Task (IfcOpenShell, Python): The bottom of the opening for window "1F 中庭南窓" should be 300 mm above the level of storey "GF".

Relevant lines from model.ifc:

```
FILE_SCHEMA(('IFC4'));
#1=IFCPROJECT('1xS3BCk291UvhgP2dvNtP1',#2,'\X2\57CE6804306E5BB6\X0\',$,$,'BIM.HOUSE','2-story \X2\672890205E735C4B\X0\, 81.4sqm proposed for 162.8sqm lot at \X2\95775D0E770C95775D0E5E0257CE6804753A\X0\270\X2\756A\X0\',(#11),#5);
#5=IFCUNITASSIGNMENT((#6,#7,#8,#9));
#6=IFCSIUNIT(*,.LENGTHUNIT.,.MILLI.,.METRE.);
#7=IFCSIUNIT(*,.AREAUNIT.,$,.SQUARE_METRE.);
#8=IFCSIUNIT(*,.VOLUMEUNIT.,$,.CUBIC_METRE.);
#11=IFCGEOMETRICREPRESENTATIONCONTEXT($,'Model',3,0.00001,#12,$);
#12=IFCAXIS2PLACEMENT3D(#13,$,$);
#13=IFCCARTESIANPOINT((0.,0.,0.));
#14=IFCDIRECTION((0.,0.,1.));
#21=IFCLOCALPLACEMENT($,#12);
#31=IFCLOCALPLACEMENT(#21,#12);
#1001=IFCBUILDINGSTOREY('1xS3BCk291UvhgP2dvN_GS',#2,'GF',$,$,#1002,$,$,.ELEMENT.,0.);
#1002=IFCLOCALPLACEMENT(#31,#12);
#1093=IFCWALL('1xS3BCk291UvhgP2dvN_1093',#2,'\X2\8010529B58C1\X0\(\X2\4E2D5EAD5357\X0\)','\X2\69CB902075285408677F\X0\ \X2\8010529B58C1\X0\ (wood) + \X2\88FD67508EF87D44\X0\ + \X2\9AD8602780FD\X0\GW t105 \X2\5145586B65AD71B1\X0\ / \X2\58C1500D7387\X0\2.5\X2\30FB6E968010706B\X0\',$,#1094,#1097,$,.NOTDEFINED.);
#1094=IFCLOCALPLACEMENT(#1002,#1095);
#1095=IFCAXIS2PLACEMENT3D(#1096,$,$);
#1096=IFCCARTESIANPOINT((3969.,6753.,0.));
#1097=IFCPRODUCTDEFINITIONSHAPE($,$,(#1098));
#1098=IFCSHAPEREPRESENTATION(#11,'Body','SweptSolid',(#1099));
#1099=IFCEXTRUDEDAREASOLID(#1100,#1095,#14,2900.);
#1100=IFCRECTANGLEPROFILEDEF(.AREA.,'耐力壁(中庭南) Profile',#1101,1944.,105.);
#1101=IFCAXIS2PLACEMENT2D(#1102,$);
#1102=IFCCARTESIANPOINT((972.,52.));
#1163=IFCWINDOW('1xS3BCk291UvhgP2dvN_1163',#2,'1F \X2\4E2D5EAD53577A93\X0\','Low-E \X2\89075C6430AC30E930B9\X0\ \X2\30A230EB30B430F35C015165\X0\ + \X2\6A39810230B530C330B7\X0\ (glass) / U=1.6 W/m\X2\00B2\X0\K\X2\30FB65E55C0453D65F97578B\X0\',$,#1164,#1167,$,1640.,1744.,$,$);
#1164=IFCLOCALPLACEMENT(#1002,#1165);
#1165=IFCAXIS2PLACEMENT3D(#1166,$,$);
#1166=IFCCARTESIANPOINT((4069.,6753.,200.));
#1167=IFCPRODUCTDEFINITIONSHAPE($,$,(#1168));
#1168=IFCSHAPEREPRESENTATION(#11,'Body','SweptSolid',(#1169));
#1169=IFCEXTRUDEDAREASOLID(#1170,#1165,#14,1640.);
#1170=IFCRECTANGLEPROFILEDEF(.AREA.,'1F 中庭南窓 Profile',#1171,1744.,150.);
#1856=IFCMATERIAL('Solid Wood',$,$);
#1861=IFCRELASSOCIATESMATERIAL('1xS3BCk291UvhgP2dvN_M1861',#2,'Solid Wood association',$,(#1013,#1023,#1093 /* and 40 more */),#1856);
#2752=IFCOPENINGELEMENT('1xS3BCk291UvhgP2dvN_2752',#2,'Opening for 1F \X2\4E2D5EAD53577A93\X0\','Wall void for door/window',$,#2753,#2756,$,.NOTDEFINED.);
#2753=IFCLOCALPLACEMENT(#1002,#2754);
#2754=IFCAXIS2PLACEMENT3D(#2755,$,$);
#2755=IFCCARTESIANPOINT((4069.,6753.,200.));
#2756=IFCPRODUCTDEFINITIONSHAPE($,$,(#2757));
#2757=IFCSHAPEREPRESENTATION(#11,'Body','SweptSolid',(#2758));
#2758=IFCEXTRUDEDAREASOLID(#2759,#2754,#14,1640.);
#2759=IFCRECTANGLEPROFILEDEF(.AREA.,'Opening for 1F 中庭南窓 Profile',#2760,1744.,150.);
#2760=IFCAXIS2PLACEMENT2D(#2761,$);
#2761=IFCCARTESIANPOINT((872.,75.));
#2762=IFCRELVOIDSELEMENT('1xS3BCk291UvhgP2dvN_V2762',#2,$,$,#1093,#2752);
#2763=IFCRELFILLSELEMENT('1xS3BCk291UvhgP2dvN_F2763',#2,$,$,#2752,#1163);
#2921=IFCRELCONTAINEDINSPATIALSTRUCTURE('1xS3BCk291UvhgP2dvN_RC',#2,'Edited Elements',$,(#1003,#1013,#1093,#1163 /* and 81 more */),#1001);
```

```python
import numpy as np
import ifcopenshell
import ifcopenshell.api.geometry
import ifcopenshell.geom
import ifcopenshell.util.element
import ifcopenshell.util.placement
import ifcopenshell.util.shape
import ifcopenshell.util.unit

model = ifcopenshell.open("model.ifc")
unit_scale = ifcopenshell.util.unit.calculate_unit_scale(model)

window = model.by_guid("1xS3BCk291UvhgP2dvN_1163")
opening = window.FillsVoids[0].RelatingOpeningElement
storey = ifcopenshell.util.element.get_container(window, ifc_class="IfcBuildingStorey")
level = ifcopenshell.util.placement.get_local_placement(storey.ObjectPlacement)[2, 3]

# The opening's origin need not be at the sill, so measure its lowest point.
shape = ifcopenshell.geom.create_shape(ifcopenshell.geom.settings(), opening)
bottom = ifcopenshell.util.shape.get_shape_bottom_elevation(shape, shape.geometry) / unit_scale
dz = level + 0.3 / unit_scale - bottom

shift = np.array([0.0, 0.0, dz])
# The window is not placed relative to its opening, so move both.
for product in (opening, window):
    matrix = ifcopenshell.util.placement.get_local_placement(product.ObjectPlacement)
    matrix[:3, 3] += shift
    ifcopenshell.api.geometry.edit_object_placement(model, product=product, matrix=matrix, is_si=False)

print(f"moved by {dz * unit_scale:+.3f} m")

model.write("model-out.ifc")
```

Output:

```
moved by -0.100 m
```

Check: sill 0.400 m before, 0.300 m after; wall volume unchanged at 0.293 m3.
